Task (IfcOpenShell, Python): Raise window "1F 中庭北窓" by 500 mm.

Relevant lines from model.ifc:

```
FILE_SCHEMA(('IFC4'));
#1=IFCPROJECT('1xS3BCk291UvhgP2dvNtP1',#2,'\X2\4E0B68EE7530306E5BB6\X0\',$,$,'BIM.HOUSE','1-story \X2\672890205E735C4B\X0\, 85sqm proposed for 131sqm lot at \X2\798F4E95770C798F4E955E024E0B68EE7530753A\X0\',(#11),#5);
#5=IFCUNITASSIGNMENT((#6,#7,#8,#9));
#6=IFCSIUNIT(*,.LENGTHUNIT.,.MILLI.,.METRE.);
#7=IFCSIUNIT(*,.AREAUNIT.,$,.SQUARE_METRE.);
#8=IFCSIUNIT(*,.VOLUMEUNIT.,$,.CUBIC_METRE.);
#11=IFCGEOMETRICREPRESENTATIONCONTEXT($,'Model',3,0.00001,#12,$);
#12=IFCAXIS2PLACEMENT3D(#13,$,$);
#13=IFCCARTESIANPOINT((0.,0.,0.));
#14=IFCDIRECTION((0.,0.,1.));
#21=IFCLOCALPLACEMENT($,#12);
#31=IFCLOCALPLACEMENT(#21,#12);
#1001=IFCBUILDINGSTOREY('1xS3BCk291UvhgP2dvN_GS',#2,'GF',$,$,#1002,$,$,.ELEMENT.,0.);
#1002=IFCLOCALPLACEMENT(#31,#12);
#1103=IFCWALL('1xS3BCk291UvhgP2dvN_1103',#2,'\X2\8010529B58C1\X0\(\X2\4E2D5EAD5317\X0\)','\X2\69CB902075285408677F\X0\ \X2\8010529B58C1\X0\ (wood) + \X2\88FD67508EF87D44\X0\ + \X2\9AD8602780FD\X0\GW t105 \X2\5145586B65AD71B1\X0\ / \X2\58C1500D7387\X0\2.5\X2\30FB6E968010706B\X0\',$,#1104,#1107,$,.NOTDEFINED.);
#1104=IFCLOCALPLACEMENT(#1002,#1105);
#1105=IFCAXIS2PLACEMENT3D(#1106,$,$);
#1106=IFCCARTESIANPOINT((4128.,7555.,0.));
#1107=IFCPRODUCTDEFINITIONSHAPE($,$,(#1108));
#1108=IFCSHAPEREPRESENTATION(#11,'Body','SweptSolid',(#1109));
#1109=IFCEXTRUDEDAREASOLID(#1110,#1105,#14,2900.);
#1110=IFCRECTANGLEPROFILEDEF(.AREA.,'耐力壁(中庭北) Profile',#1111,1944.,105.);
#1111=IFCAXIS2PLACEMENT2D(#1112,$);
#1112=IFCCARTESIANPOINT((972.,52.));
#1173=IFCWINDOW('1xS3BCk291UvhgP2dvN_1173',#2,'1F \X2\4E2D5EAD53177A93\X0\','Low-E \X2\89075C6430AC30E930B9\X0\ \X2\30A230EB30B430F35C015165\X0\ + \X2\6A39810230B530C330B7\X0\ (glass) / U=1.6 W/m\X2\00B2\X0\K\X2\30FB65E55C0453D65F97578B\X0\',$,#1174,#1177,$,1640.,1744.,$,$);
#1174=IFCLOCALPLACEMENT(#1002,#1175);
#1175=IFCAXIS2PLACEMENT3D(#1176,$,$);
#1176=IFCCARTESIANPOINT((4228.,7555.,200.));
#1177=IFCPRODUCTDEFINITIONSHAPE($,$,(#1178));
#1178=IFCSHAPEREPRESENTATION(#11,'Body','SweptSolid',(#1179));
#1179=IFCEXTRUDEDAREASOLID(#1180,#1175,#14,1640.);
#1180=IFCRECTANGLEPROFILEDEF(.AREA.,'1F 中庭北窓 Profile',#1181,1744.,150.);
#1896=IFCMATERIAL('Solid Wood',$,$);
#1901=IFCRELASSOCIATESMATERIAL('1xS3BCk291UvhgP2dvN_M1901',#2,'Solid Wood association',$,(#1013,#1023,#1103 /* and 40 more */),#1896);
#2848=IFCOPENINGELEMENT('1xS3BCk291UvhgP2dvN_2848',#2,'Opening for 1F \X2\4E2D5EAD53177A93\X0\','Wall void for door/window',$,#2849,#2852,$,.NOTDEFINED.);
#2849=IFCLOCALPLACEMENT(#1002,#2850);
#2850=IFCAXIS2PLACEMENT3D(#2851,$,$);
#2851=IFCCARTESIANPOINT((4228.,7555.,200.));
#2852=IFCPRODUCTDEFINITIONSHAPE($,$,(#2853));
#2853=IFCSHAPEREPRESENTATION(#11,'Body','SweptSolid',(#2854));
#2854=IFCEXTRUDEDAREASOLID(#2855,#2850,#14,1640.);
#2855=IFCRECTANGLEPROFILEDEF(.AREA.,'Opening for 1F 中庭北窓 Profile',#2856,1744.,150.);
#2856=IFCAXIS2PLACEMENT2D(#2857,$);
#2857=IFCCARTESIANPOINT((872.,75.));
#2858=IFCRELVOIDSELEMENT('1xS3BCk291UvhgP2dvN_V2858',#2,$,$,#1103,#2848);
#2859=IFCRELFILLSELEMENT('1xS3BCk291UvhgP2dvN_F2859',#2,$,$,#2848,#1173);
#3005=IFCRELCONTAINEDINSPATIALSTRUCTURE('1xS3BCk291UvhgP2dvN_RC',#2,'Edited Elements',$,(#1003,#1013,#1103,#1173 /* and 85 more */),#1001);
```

```python
import numpy as np
import ifcopenshell
import ifcopenshell.api.geometry
import ifcopenshell.util.placement
import ifcopenshell.util.unit

model = ifcopenshell.open("model.ifc")
unit_scale = ifcopenshell.util.unit.calculate_unit_scale(model)

window = model.by_id(1173)
opening = window.FillsVoids[0].RelatingOpeningElement
dz = 0.5 / unit_scale

shift = np.array([0.0, 0.0, dz])
# The window is not placed relative to its opening, so move both.
for product in (opening, window):
    matrix = ifcopenshell.util.placement.get_local_placement(product.ObjectPlacement)
    matrix[:3, 3] += shift
    ifcopenshell.api.geometry.edit_object_placement(model, product=product, matrix=matrix, is_si=False)

print(f"moved by {dz * unit_scale:+.3f} m")

model.write("model-out.ifc")
```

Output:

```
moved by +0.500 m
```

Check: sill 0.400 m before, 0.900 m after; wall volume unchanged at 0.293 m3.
